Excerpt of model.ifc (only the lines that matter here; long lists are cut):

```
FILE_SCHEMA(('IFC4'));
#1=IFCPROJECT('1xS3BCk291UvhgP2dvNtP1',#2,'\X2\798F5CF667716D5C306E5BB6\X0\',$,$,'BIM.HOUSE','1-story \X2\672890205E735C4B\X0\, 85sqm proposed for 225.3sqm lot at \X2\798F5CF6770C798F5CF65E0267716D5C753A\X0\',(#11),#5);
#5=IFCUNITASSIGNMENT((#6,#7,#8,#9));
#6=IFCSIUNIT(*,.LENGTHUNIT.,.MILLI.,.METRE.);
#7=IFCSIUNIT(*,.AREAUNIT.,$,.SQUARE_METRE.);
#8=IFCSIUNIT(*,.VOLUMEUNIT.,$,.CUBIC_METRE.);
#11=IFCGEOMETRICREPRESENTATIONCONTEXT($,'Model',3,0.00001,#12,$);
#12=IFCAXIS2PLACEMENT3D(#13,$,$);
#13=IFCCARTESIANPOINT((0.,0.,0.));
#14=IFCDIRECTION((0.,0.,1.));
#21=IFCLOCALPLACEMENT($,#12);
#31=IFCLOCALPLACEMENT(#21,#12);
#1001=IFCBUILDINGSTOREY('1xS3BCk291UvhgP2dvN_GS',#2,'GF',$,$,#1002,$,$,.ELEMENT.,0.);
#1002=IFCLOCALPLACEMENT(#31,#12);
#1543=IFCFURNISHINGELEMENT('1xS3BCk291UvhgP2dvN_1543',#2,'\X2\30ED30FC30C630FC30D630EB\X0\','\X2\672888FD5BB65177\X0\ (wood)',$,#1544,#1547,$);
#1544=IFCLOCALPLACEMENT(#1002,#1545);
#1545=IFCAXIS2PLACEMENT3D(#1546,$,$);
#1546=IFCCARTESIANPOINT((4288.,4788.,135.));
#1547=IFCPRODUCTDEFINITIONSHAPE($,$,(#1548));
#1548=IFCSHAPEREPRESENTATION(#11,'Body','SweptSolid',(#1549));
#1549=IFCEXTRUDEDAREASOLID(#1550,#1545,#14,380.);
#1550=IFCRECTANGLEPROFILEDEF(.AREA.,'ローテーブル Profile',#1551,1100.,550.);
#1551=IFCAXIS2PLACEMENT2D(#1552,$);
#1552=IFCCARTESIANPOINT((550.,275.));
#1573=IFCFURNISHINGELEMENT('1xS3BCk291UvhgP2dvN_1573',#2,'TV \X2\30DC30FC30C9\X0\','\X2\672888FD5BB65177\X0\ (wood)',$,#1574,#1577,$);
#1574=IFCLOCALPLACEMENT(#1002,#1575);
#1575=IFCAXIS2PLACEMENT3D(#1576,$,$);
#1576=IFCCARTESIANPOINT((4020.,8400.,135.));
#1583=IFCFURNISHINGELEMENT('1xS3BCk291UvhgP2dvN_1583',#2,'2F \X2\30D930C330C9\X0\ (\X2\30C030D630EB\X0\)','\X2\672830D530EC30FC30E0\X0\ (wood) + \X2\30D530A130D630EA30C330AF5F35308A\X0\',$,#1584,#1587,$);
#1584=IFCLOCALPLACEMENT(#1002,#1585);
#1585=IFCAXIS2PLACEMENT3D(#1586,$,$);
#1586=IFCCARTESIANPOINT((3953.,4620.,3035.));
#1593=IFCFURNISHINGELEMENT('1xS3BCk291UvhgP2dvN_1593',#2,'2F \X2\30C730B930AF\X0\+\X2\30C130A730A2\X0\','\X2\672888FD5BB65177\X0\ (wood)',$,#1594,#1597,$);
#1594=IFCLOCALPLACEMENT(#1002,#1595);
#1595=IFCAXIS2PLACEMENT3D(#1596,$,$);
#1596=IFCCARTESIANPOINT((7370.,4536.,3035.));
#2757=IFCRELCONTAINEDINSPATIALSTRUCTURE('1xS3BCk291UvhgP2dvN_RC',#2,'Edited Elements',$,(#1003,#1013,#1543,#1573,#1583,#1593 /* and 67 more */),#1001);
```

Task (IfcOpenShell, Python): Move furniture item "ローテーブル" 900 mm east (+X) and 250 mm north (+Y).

```python
import ifcopenshell
import ifcopenshell.api.geometry
import ifcopenshell.util.placement
import ifcopenshell.util.unit

model = ifcopenshell.open("model.ifc")
unit_scale = ifcopenshell.util.unit.calculate_unit_scale(model)

item = model.by_guid("1xS3BCk291UvhgP2dvN_1543")
matrix = ifcopenshell.util.placement.get_local_placement(item.ObjectPlacement)
matrix[0, 3] += 0.9 / unit_scale
matrix[1, 3] += 0.25 / unit_scale
ifcopenshell.api.geometry.edit_object_placement(model, product=item, matrix=matrix, is_si=False)

print(ifcopenshell.util.placement.get_local_placement(item.ObjectPlacement).round(3) + 0.0)

model.write("model-out.ifc")
```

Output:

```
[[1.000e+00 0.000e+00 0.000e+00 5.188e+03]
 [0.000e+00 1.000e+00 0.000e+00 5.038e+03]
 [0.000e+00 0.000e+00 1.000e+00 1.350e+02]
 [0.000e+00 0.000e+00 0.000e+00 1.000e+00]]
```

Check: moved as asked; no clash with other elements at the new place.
